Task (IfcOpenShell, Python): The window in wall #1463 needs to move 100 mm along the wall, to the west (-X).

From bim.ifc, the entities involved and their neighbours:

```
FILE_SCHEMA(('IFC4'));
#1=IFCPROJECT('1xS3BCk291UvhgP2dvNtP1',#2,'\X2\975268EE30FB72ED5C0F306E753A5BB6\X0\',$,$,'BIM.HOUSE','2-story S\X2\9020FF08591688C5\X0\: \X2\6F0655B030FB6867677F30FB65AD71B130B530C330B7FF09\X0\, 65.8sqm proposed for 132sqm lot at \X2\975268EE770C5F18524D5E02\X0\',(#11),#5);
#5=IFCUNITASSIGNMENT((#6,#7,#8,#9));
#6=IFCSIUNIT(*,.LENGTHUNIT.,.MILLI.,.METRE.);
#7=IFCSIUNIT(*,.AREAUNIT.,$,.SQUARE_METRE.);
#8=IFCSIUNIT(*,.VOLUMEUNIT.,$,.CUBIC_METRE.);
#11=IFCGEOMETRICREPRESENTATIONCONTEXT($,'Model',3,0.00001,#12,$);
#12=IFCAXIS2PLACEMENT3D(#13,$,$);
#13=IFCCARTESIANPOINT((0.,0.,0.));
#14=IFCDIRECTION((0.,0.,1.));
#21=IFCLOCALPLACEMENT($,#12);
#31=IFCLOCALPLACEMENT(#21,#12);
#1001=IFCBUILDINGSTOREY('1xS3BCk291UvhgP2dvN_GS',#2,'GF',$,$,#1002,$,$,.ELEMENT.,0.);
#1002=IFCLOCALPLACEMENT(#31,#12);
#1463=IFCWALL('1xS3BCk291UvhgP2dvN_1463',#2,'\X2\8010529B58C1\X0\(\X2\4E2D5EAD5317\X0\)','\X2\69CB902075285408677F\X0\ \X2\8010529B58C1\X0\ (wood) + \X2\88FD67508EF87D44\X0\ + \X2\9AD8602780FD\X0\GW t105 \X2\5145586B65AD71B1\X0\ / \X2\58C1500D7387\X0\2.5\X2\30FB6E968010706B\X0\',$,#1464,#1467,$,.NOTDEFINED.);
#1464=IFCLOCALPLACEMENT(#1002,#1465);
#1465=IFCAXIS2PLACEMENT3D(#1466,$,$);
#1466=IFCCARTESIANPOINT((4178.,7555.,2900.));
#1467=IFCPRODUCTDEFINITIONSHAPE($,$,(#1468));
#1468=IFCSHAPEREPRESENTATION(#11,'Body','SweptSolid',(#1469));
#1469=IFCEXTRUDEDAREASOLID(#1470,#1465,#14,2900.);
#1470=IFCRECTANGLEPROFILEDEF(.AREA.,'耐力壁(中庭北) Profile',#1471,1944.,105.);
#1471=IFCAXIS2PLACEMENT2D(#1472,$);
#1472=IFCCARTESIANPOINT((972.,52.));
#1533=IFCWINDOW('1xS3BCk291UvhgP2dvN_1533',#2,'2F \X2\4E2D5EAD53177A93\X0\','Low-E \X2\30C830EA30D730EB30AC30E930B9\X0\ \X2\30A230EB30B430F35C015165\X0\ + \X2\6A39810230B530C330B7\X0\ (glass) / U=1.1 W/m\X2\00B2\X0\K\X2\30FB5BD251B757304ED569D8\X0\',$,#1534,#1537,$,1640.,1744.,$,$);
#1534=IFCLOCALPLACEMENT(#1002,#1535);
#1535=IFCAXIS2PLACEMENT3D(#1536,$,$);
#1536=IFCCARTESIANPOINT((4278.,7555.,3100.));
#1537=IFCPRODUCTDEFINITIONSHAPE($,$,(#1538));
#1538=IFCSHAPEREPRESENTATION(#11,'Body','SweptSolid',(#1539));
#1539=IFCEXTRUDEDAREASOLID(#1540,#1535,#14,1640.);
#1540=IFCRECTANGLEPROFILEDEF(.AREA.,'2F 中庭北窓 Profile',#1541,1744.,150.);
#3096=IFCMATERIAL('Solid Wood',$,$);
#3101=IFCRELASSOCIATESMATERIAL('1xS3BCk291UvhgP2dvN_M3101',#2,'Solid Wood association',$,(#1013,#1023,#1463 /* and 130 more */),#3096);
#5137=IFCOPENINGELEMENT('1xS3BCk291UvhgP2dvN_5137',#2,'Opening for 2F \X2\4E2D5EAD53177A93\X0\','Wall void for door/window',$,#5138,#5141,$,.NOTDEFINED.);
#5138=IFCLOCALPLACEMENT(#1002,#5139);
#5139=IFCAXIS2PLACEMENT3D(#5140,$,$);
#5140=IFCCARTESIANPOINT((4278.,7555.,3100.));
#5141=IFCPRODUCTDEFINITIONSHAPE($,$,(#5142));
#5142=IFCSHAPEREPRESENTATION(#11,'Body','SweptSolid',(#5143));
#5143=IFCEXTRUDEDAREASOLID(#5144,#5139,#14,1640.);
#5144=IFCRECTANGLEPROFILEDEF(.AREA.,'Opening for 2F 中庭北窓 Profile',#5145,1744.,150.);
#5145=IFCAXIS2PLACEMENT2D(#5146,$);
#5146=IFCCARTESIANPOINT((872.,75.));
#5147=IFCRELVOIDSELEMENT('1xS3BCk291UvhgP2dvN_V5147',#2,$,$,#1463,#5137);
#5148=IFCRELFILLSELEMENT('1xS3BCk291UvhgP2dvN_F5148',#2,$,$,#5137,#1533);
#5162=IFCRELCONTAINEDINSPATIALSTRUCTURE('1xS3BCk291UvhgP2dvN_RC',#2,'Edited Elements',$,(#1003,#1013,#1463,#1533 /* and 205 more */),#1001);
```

```python
import ifcopenshell
import ifcopenshell.api.geometry
import ifcopenshell.util.placement
import ifcopenshell.util.unit

model = ifcopenshell.open("bim.ifc")
unit_scale = ifcopenshell.util.unit.calculate_unit_scale(model)

window = model.by_guid("1xS3BCk291UvhgP2dvN_1533")
opening = window.FillsVoids[0].RelatingOpeningElement
wall = opening.VoidsElements[0].RelatingBuildingElement

wall_matrix = ifcopenshell.util.placement.get_local_placement(wall.ObjectPlacement)
shift = wall_matrix[:3, 0] * -0.1 / unit_scale
before = ifcopenshell.util.placement.get_local_placement(window.ObjectPlacement)[:3, 3].copy()

# The window is not placed relative to its opening, so move both.
for product in (opening, window):
    matrix = ifcopenshell.util.placement.get_local_placement(product.ObjectPlacement)
    matrix[:3, 3] += shift
    ifcopenshell.api.geometry.edit_object_placement(model, product=product, matrix=matrix, is_si=False)

after = ifcopenshell.util.placement.get_local_placement(window.ObjectPlacement)[:3, 3]
print("window moved by", (after - before).round(3) + 0.0)

model.write("bim-out.ifc")
```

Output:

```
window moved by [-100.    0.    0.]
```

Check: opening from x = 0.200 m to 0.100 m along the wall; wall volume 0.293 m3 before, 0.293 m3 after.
